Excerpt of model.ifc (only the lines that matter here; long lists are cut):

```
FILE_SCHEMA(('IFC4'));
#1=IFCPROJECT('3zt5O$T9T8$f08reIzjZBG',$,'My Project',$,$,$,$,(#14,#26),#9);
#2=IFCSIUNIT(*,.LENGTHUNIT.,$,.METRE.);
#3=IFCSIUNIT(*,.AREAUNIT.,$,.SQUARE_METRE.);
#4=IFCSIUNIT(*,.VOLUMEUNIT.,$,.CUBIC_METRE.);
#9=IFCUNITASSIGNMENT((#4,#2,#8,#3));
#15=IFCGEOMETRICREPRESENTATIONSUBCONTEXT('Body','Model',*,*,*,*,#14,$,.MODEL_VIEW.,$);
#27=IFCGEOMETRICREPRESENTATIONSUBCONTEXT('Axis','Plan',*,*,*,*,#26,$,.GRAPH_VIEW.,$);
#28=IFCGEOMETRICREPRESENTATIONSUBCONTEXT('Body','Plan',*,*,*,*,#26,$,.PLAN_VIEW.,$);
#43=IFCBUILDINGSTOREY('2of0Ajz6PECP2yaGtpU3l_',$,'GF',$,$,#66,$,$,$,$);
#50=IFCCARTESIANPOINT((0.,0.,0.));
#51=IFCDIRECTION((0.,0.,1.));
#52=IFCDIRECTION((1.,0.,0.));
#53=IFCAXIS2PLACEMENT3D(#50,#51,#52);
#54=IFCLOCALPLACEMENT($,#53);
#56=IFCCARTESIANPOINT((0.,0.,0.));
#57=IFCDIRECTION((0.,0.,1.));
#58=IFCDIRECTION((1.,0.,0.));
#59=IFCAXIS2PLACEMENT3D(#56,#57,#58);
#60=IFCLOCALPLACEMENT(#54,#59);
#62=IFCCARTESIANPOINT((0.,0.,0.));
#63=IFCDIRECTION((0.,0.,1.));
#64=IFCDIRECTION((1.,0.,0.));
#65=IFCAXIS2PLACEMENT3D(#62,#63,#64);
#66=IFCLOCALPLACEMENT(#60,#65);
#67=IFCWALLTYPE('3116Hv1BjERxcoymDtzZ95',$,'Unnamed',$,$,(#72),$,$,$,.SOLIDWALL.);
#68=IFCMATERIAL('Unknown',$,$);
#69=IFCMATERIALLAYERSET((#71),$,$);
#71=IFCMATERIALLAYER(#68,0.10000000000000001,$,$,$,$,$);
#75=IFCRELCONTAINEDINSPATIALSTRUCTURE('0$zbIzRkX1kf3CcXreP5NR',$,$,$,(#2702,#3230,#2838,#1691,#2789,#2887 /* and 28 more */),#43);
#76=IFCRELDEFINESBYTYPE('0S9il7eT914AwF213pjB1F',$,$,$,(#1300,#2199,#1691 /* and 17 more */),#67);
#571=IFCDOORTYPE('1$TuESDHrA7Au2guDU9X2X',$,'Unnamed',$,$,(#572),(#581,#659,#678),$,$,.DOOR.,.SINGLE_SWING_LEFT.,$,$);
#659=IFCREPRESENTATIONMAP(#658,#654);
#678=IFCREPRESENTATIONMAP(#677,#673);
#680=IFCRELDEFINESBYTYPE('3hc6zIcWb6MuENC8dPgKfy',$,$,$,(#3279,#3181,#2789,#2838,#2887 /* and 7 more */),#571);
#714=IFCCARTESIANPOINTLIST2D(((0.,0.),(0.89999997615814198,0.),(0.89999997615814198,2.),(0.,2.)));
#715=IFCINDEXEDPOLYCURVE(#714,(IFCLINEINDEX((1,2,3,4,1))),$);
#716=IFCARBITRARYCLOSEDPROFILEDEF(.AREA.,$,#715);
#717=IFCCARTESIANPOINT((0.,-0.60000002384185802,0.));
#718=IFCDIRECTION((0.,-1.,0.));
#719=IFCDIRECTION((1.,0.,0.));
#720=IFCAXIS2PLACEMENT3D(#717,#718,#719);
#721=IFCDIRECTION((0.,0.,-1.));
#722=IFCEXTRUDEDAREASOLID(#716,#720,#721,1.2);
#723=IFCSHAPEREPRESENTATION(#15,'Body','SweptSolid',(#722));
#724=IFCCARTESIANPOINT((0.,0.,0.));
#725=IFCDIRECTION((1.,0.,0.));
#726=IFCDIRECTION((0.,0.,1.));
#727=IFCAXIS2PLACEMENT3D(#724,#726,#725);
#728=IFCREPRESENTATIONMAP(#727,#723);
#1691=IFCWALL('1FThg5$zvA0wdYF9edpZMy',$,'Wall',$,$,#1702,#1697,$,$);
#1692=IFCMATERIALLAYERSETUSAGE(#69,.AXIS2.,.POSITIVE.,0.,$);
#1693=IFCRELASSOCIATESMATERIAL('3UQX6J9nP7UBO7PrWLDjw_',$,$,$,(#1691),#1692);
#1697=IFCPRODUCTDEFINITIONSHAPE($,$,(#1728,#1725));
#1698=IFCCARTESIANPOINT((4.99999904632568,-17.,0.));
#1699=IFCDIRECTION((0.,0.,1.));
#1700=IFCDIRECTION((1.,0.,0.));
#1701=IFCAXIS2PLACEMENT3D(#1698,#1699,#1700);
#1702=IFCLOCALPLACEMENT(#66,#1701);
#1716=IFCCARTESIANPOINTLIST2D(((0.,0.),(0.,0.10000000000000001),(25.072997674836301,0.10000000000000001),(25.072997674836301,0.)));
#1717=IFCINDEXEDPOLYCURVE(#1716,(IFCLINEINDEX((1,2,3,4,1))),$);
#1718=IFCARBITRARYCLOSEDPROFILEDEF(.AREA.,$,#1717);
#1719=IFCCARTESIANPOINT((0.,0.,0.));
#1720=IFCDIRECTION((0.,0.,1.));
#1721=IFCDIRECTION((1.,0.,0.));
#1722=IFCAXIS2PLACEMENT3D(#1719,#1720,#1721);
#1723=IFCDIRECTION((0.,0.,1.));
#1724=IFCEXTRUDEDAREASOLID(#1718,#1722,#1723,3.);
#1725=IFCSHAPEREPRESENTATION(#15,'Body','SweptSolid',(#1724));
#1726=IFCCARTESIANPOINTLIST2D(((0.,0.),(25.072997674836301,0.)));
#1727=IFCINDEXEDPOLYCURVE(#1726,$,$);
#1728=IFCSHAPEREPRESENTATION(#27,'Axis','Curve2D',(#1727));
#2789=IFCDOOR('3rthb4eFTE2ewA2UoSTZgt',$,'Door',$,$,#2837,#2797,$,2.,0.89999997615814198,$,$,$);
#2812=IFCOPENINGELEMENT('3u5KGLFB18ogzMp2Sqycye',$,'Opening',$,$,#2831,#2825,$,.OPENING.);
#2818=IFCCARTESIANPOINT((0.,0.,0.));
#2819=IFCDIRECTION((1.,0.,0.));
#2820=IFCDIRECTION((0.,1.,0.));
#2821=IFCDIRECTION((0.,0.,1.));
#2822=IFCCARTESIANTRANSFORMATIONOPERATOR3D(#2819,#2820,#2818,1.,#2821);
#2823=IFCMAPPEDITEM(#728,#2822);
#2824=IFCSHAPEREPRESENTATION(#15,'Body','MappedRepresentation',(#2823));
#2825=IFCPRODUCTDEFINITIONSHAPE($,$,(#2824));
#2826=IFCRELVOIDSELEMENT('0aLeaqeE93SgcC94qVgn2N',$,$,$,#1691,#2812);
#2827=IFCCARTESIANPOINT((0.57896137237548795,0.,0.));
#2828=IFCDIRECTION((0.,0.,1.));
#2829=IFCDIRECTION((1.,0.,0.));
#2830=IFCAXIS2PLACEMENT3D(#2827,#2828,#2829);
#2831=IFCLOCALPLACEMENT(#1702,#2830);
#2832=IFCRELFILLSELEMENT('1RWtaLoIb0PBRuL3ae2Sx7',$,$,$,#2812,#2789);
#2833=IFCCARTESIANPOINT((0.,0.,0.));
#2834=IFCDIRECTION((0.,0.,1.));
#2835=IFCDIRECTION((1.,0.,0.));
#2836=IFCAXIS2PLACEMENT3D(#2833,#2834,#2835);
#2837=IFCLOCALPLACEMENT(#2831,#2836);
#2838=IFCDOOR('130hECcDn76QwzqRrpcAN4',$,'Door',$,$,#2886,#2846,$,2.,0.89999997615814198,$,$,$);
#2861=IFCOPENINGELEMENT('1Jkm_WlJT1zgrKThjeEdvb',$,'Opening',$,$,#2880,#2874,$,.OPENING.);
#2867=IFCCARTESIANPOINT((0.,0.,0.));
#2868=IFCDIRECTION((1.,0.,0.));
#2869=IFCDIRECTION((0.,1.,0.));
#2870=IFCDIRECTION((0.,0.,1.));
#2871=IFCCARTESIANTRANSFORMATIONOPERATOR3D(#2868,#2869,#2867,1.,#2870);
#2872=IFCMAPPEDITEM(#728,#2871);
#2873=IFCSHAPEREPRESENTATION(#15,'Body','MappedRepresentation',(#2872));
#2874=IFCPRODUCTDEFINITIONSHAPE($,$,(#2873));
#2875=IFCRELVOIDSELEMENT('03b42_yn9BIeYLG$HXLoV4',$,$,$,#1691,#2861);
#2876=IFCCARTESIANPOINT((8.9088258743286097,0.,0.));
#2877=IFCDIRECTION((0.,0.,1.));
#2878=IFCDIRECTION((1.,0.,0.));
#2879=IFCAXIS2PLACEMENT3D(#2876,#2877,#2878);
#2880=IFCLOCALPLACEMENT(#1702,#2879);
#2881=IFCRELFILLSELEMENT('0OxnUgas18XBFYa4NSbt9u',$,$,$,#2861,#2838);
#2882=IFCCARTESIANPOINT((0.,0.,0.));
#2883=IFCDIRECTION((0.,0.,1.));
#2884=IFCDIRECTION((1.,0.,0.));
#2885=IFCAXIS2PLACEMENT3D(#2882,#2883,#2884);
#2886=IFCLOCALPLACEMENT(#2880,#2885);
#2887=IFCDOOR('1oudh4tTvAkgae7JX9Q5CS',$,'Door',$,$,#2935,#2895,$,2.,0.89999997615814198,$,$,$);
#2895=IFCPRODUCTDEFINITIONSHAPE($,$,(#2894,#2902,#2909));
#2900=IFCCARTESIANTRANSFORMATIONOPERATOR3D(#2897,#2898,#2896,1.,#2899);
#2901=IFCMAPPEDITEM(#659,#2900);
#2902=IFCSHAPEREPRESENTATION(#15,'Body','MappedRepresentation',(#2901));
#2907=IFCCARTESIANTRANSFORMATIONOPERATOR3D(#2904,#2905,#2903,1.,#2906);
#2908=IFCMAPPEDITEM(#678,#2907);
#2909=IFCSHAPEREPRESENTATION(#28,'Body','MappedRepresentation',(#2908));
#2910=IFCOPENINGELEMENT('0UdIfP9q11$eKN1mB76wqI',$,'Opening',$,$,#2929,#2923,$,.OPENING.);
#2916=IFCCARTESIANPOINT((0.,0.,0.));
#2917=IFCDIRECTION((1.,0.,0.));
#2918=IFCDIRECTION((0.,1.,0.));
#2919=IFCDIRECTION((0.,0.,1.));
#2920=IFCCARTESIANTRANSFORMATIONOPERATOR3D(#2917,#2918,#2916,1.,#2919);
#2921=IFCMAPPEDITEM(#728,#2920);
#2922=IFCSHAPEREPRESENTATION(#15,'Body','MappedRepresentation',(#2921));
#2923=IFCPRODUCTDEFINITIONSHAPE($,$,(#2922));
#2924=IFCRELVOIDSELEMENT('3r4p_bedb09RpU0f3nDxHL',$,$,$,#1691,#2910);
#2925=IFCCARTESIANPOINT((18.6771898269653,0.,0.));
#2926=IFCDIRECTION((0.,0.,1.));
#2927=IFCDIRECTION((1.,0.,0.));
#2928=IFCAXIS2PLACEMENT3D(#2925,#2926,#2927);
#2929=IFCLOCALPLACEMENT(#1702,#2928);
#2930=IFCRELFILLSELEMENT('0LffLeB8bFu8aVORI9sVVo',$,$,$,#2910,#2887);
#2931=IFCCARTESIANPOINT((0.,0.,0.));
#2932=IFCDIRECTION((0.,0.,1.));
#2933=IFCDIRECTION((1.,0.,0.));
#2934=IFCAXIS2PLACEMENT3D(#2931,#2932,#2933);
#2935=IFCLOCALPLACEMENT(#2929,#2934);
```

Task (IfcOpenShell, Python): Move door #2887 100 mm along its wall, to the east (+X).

```python
import ifcopenshell
import ifcopenshell.api.geometry
import ifcopenshell.util.placement

model = ifcopenshell.open("model.ifc")

door = model.by_id(2887)
opening = door.FillsVoids[0].RelatingOpeningElement
wall = opening.VoidsElements[0].RelatingBuildingElement

wall_matrix = ifcopenshell.util.placement.get_local_placement(wall.ObjectPlacement)
shift = wall_matrix[:3, 0] * 0.1
before = ifcopenshell.util.placement.get_local_placement(door.ObjectPlacement)[:3, 3].copy()

# The door is placed relative to its opening, so it follows when the opening moves.
matrix = ifcopenshell.util.placement.get_local_placement(opening.ObjectPlacement)
matrix[:3, 3] += shift
ifcopenshell.api.geometry.edit_object_placement(
    model, product=opening, matrix=matrix, is_si=False, should_transform_children=True
)

after = ifcopenshell.util.placement.get_local_placement(door.ObjectPlacement)[:3, 3]
print("door moved by", (after - before).round(3) + 0.0)

model.write("model_updated.ifc")
```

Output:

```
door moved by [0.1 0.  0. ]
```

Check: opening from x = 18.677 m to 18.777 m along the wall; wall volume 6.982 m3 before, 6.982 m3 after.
